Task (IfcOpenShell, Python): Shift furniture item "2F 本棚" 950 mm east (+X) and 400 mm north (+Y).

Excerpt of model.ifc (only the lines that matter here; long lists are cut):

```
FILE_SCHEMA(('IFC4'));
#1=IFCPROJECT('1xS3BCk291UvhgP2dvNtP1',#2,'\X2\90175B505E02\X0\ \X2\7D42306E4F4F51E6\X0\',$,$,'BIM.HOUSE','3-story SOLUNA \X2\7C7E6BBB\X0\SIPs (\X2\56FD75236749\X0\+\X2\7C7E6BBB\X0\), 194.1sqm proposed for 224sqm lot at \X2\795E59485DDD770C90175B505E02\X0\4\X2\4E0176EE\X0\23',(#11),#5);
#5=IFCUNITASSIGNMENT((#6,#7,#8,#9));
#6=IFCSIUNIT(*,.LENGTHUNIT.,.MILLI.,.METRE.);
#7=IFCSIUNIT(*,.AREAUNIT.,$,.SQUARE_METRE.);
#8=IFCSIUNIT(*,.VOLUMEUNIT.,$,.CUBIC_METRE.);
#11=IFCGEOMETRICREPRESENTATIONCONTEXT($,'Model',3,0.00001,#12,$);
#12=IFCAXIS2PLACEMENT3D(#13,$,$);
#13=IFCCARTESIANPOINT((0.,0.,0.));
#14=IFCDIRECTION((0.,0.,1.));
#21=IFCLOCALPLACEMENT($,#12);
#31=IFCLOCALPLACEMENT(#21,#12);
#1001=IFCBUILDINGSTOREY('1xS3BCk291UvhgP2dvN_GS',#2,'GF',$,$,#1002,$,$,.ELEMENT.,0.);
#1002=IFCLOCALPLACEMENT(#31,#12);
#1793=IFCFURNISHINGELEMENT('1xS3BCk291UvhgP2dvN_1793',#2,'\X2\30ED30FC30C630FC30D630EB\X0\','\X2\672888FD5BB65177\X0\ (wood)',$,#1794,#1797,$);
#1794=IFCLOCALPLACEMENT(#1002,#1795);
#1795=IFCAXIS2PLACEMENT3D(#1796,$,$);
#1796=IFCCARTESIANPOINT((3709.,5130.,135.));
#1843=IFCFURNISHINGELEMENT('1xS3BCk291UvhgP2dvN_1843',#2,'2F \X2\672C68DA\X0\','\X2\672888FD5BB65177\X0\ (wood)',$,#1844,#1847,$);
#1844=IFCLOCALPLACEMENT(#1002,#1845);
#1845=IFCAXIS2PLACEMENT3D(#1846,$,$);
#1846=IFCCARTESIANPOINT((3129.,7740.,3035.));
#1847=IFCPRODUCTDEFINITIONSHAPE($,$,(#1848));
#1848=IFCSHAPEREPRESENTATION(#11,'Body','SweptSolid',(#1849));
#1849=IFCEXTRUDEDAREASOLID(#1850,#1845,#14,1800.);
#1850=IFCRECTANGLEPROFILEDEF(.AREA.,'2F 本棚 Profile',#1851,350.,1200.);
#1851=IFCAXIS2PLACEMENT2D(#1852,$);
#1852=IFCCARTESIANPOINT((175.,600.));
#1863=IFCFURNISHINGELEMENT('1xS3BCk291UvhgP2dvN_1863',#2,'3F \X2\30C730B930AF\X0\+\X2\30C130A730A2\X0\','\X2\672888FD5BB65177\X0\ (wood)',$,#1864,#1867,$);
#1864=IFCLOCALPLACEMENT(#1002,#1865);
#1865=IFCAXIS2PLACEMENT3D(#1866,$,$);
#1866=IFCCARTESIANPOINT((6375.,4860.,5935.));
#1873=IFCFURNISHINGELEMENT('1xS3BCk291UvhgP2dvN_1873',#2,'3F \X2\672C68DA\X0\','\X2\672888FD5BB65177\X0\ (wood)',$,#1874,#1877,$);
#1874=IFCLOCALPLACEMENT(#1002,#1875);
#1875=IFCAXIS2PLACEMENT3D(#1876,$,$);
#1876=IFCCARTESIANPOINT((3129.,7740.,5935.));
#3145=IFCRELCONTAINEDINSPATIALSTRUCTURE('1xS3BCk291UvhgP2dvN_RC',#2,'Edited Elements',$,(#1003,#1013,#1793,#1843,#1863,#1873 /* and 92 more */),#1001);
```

```python
import ifcopenshell
import ifcopenshell.api.geometry
import ifcopenshell.util.placement
import ifcopenshell.util.unit

model = ifcopenshell.open("model.ifc")
unit_scale = ifcopenshell.util.unit.calculate_unit_scale(model)

item = model.by_guid("1xS3BCk291UvhgP2dvN_1843")
matrix = ifcopenshell.util.placement.get_local_placement(item.ObjectPlacement)
matrix[0, 3] += 0.95 / unit_scale
matrix[1, 3] += 0.4 / unit_scale
ifcopenshell.api.geometry.edit_object_placement(model, product=item, matrix=matrix, is_si=False)

print(ifcopenshell.util.placement.get_local_placement(item.ObjectPlacement).round(3) + 0.0)

model.write("model_edited.ifc")
```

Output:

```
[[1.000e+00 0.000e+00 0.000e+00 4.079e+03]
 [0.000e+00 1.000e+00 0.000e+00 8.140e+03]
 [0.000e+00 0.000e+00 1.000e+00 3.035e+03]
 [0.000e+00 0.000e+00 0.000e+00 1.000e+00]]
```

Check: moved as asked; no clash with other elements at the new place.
